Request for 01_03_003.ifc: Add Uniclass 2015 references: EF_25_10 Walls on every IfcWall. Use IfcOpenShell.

First a look at what the model holds.

```python
import ifcopenshell

model = ifcopenshell.open("01_03_003.ifc")
print(model.schema)
print("classifications:", [c.Name for c in model.by_type("IfcClassification")])
for ifc_class in ("IfcDoor", "IfcRoof", "IfcStair", "IfcWall", "IfcWindow"):
    print(ifc_class, len(model.by_type(ifc_class)))
```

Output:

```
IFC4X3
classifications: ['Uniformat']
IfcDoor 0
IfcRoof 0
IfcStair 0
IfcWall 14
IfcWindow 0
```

```python
import ifcopenshell
import ifcopenshell.api.classification

model = ifcopenshell.open("01_03_003.ifc")

system = ifcopenshell.api.classification.add_classification(model, classification="Uniclass 2015")

codes = {
    "IfcWall": ("EF_25_10", "Walls"),
}
for ifc_class, (code, name) in codes.items():
    products = model.by_type(ifc_class)
    ifcopenshell.api.classification.add_reference(
        model, products=products, classification=system, identification=code, name=name
    )
    print(code, len(products))

model.write("01_03_003_updated.ifc")
```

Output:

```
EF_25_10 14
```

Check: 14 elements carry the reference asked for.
